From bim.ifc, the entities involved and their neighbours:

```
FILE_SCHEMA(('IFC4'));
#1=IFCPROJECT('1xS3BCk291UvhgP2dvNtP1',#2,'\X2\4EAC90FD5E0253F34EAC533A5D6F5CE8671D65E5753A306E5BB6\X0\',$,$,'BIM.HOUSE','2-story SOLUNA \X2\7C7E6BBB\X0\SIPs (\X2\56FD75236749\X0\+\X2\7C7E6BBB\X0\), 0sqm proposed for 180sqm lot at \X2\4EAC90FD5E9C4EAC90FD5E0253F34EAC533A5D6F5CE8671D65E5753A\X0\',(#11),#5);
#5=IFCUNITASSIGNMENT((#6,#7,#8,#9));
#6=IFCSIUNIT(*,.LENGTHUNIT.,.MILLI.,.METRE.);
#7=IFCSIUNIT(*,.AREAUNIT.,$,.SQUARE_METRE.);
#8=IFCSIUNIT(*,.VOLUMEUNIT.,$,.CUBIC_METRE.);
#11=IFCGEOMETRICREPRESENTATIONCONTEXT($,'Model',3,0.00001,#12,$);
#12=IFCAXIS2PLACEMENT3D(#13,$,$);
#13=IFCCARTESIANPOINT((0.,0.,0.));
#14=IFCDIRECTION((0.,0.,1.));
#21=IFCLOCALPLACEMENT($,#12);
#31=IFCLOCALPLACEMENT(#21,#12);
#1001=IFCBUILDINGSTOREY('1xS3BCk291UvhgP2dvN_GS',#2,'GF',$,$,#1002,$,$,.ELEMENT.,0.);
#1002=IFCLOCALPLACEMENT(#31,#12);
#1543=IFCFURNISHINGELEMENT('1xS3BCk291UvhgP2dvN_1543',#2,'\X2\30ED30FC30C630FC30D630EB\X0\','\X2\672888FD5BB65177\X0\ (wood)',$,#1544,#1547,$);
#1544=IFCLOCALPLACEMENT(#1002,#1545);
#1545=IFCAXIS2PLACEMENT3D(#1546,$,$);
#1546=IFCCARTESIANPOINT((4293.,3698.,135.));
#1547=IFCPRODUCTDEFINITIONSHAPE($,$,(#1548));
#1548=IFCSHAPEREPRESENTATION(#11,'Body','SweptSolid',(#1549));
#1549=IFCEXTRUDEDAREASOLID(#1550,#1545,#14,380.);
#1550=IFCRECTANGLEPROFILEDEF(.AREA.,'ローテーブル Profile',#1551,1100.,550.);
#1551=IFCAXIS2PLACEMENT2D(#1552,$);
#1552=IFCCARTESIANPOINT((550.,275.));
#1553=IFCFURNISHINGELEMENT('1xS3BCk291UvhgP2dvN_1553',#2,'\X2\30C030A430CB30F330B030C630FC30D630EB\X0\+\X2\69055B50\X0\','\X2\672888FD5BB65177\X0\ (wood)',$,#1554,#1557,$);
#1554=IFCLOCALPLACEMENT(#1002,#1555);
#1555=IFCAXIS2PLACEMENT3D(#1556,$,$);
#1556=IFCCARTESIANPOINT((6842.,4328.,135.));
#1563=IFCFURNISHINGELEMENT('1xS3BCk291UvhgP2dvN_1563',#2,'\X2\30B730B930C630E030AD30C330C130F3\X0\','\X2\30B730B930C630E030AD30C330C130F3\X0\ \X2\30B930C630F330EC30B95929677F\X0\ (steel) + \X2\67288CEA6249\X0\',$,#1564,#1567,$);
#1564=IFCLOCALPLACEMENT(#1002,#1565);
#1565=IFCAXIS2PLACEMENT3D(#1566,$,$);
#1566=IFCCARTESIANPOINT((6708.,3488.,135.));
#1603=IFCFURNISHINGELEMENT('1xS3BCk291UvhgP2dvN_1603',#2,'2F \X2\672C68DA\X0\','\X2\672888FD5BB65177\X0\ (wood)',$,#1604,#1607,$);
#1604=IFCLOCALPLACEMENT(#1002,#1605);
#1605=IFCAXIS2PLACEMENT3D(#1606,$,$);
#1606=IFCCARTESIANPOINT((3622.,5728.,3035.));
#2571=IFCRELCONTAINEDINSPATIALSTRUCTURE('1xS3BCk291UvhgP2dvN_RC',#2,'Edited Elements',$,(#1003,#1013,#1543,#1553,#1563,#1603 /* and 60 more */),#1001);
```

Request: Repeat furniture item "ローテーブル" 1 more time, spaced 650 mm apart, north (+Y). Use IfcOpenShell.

```python
import numpy as np
import ifcopenshell
import ifcopenshell.api.geometry
import ifcopenshell.api.root
import ifcopenshell.util.element
import ifcopenshell.util.placement
import ifcopenshell.util.unit

model = ifcopenshell.open("bim.ifc")
unit_scale = ifcopenshell.util.unit.calculate_unit_scale(model)


def reuse_history(source, copy):
    """copy_class also copies each property set's owner history, people and application; keep the originals."""
    for rel in copy.IsDefinedBy:
        if rel.is_a("IfcRelDefinesByProperties") and (history := rel.RelatingPropertyDefinition.OwnerHistory):
            rel.RelatingPropertyDefinition.OwnerHistory = source.OwnerHistory
            ifcopenshell.util.element.remove_deep2(model, history)


source = model.by_guid("1xS3BCk291UvhgP2dvN_1543")
base = ifcopenshell.util.placement.get_local_placement(source.ObjectPlacement)
step = np.array([0.0, 1.0, 0.0]) * 0.65 / unit_scale

for i in range(1, 2):
    copy = ifcopenshell.api.root.copy_class(model, product=source)
    copy.Representation = ifcopenshell.util.element.copy_deep(
        model, source.Representation, exclude=["IfcGeometricRepresentationContext", "IfcRepresentationMap"]
    )
    reuse_history(source, copy)
    matrix = base.copy()
    matrix[:3, 3] += i * step
    print("added at", matrix[:3, 3].round(3) + 0.0)
    ifcopenshell.api.geometry.edit_object_placement(model, product=copy, matrix=matrix, is_si=False)

model.write("bim_updated.ifc")
```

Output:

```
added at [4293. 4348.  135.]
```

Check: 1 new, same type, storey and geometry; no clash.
